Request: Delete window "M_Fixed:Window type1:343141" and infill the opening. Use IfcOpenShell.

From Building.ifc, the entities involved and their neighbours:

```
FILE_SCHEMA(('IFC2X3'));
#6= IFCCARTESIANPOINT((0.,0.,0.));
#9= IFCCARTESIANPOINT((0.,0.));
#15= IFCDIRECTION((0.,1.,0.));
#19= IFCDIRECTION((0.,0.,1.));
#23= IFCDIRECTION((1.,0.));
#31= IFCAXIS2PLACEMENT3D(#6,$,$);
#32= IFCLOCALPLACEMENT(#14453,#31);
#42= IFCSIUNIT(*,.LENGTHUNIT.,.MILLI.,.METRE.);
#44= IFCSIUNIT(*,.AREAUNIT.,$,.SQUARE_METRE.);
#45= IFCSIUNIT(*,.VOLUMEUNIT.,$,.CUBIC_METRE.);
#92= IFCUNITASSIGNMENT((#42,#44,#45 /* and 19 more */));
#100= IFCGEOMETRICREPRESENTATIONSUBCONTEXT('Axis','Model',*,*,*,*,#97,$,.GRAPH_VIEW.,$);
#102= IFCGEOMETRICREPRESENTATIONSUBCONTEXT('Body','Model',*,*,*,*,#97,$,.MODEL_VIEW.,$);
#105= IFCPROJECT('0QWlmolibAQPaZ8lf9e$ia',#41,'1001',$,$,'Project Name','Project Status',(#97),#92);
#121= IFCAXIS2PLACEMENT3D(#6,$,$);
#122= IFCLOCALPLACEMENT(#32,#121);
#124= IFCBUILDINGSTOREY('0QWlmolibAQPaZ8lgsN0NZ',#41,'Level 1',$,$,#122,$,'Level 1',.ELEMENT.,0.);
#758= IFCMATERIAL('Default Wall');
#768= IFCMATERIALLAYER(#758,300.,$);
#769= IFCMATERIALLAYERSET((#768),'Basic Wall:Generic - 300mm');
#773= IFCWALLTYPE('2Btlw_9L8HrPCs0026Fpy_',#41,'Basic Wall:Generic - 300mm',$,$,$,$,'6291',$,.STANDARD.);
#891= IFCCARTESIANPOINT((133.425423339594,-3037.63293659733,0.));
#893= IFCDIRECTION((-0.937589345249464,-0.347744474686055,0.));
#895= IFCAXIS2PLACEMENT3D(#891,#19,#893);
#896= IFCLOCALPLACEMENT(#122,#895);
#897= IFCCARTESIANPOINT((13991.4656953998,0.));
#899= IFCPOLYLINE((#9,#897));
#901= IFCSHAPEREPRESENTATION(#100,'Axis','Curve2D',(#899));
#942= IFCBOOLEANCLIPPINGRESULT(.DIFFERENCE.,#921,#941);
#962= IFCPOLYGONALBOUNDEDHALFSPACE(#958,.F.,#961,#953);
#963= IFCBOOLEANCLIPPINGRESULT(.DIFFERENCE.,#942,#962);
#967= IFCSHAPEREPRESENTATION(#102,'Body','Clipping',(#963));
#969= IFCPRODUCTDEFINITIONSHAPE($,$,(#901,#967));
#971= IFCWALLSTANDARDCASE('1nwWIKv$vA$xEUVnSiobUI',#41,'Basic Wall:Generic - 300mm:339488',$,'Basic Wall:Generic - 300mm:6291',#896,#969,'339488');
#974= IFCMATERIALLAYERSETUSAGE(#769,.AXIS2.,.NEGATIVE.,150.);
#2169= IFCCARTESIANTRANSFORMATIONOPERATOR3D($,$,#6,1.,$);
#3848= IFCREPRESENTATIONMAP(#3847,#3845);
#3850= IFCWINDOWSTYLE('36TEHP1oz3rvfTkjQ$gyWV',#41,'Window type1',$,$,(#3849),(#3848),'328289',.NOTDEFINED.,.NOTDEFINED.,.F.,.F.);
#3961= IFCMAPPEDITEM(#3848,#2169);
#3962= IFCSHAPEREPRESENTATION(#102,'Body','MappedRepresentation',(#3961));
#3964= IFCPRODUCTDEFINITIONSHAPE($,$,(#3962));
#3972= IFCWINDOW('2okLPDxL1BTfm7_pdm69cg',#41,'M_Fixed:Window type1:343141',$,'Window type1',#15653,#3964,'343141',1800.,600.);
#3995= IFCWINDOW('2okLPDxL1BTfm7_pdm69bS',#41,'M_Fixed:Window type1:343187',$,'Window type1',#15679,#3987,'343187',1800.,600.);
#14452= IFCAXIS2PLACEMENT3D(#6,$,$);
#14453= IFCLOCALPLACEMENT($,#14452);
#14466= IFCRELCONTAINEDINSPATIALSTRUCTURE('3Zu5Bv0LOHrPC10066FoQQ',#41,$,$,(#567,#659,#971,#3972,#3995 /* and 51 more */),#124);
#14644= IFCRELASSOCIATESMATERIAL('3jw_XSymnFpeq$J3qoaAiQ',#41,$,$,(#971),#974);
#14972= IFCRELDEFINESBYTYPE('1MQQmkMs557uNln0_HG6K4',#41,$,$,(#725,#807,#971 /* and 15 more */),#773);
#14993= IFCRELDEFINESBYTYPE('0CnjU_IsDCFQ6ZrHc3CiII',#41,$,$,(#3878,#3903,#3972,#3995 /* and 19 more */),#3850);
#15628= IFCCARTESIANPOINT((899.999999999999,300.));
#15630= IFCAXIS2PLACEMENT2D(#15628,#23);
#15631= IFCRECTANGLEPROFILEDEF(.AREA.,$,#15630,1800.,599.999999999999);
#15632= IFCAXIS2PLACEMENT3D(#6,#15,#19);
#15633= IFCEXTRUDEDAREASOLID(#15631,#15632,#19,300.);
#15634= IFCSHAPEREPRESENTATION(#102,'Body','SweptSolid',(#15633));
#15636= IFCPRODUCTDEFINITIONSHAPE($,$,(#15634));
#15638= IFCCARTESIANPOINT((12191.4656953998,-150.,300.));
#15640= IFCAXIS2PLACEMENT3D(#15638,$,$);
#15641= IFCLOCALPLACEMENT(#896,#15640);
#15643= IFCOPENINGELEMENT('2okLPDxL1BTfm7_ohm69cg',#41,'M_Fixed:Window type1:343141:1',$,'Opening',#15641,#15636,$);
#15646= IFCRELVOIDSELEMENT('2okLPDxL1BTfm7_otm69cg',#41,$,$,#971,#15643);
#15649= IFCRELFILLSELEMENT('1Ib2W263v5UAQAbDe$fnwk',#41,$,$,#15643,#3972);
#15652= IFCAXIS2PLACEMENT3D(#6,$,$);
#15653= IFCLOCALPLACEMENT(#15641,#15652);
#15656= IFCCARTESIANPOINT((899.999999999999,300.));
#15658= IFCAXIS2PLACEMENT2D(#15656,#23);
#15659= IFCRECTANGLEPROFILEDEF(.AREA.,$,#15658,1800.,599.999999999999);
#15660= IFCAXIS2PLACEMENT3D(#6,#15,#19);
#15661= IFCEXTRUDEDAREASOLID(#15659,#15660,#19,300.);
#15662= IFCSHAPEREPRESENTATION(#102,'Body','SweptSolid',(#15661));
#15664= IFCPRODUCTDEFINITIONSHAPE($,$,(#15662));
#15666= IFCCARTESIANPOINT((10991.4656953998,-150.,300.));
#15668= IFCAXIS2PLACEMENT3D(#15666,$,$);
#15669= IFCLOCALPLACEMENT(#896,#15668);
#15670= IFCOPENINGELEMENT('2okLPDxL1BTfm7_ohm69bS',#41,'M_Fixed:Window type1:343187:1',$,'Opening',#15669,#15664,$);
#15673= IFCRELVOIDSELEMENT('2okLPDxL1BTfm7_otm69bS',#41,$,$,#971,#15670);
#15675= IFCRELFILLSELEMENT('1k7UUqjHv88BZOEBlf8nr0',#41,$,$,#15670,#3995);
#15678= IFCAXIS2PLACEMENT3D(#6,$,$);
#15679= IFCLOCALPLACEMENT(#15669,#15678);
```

```python
import ifcopenshell
import ifcopenshell.api.feature
import ifcopenshell.api.root
import ifcopenshell.geom
import ifcopenshell.util.shape

model = ifcopenshell.open("Building.ifc")
settings = ifcopenshell.geom.settings()


def volume(element):
    """Net volume in cubic metres, openings subtracted."""
    shape = ifcopenshell.geom.create_shape(settings, element)
    return ifcopenshell.util.shape.get_volume(shape.geometry)


window = model.by_guid("2okLPDxL1BTfm7_pdm69cg")
opening = window.FillsVoids[0].RelatingOpeningElement
wall = opening.VoidsElements[0].RelatingBuildingElement
before = volume(wall)

ifcopenshell.api.root.remove_product(model, product=window)
ifcopenshell.api.feature.remove_feature(model, feature=opening)

after = volume(wall)

print(f"wall volume {before:.3f} -> {after:.3f} m3")

model.write("Building-out.ifc")
```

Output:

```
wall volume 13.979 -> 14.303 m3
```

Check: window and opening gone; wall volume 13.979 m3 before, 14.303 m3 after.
